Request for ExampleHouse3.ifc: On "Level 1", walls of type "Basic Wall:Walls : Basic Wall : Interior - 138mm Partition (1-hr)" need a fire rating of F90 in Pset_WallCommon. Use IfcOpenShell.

First a look at what the model holds.

```python
import ifcopenshell
import ifcopenshell.util.element

model = ifcopenshell.open("ExampleHouse3.ifc")
print(model.schema)
storey = next(s for s in model.by_type("IfcBuildingStorey") if s.Name == "Level 1")
walls = [e for e in ifcopenshell.util.element.get_decomposition(storey) if e.is_a("IfcWall")]
seen = {}
for e in walls:
    element_type = ifcopenshell.util.element.get_type(e)
    key = (element_type.Name if element_type != e and element_type else None, ifcopenshell.util.element.get_pset(e, "Pset_WallCommon", "FireRating"))
    seen[key] = seen.get(key, 0) + 1
for (name, value), count in sorted(seen.items(), key=str):
    print(count, "x", name, "|", value)
```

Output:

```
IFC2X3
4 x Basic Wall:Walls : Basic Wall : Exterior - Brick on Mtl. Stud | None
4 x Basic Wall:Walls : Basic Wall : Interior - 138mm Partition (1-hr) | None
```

```python
import ifcopenshell
import ifcopenshell.api.pset
import ifcopenshell.util.element

model = ifcopenshell.open("ExampleHouse3.ifc")

storey = next(s for s in model.by_type("IfcBuildingStorey") if s.Name == "Level 1")
walls = [e for e in ifcopenshell.util.element.get_decomposition(storey) if e.is_a("IfcWall")]

count = 0
for e in walls:
    element_type = ifcopenshell.util.element.get_type(e)
    if element_type in (None, e) or element_type.Name != "Basic Wall:Walls : Basic Wall : Interior - 138mm Partition (1-hr)":
        continue
    # add_pset returns the element's existing set when there is one.
    pset = ifcopenshell.api.pset.add_pset(model, product=e, name="Pset_WallCommon")
    ifcopenshell.api.pset.edit_pset(model, pset=pset, properties={"FireRating": "F90"})
    count += 1

print(count, "walls updated")

model.write("ExampleHouse3-out.ifc")
```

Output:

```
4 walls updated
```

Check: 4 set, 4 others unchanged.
